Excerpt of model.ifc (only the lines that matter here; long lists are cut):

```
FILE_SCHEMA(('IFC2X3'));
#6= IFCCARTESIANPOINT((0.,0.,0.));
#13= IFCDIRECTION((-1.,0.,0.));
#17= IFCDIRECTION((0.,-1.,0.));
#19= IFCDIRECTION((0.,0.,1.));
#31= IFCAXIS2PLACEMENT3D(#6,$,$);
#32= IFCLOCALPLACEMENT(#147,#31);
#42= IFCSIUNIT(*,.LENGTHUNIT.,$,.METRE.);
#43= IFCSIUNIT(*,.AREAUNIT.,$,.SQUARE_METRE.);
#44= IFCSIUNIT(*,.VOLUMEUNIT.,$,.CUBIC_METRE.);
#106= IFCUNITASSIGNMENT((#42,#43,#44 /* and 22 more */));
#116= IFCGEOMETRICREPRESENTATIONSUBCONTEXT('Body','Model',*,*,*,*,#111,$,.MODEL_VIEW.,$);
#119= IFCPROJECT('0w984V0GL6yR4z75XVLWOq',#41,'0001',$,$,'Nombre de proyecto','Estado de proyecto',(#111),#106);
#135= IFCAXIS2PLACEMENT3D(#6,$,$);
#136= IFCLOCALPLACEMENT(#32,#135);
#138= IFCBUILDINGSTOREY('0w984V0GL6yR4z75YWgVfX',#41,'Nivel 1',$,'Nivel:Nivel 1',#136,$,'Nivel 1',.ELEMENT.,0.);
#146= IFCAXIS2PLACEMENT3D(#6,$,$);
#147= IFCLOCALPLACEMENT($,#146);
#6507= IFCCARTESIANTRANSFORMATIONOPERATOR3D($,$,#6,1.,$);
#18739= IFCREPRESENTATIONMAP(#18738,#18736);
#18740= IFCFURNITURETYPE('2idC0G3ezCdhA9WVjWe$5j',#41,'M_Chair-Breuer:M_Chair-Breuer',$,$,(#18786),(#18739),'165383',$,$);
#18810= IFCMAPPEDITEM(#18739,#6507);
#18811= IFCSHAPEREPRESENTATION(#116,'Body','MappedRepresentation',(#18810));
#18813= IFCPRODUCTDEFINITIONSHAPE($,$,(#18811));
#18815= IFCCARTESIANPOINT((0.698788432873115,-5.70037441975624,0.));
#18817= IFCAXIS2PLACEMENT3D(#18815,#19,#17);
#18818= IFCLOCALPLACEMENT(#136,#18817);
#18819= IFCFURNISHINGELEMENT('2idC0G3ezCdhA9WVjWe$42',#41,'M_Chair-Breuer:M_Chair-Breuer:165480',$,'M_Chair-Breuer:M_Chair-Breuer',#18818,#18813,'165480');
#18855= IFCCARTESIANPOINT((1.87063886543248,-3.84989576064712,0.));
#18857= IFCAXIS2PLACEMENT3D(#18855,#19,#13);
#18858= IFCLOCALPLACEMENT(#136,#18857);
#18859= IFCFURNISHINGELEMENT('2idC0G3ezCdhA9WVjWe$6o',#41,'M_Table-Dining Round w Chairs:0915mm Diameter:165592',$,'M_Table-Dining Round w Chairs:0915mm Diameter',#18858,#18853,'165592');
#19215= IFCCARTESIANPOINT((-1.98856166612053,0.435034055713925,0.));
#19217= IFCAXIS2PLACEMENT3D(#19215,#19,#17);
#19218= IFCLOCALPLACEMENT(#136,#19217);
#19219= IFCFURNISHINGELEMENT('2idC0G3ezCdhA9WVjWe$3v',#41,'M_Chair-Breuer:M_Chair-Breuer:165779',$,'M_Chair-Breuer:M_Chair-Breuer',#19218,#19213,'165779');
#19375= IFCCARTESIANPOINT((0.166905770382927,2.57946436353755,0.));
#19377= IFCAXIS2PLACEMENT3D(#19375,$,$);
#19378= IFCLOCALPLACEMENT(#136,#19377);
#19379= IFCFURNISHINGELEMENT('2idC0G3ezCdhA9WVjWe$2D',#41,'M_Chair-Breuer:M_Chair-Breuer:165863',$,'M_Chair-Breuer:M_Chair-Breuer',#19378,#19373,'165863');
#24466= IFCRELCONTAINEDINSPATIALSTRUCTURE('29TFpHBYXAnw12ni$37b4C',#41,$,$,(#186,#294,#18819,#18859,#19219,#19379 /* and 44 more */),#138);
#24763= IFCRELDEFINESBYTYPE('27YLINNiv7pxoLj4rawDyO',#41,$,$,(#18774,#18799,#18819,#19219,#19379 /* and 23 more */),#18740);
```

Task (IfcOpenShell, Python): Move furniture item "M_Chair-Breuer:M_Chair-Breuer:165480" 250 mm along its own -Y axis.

```python
import ifcopenshell
import ifcopenshell.api.geometry
import ifcopenshell.util.placement
import ifcopenshell.util.unit

model = ifcopenshell.open("model.ifc")
unit_scale = ifcopenshell.util.unit.calculate_unit_scale(model)

item = model.by_guid("2idC0G3ezCdhA9WVjWe$42")
matrix = ifcopenshell.util.placement.get_local_placement(item.ObjectPlacement)
matrix[:3, 3] -= matrix[:3, 1] * 0.25 / unit_scale
ifcopenshell.api.geometry.edit_object_placement(model, product=item, matrix=matrix, is_si=False)

print(ifcopenshell.util.placement.get_local_placement(item.ObjectPlacement).round(3) + 0.0)

model.write("model_rev.ifc")
```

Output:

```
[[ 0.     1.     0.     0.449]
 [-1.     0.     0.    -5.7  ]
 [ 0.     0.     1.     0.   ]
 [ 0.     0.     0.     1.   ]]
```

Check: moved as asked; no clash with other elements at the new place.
